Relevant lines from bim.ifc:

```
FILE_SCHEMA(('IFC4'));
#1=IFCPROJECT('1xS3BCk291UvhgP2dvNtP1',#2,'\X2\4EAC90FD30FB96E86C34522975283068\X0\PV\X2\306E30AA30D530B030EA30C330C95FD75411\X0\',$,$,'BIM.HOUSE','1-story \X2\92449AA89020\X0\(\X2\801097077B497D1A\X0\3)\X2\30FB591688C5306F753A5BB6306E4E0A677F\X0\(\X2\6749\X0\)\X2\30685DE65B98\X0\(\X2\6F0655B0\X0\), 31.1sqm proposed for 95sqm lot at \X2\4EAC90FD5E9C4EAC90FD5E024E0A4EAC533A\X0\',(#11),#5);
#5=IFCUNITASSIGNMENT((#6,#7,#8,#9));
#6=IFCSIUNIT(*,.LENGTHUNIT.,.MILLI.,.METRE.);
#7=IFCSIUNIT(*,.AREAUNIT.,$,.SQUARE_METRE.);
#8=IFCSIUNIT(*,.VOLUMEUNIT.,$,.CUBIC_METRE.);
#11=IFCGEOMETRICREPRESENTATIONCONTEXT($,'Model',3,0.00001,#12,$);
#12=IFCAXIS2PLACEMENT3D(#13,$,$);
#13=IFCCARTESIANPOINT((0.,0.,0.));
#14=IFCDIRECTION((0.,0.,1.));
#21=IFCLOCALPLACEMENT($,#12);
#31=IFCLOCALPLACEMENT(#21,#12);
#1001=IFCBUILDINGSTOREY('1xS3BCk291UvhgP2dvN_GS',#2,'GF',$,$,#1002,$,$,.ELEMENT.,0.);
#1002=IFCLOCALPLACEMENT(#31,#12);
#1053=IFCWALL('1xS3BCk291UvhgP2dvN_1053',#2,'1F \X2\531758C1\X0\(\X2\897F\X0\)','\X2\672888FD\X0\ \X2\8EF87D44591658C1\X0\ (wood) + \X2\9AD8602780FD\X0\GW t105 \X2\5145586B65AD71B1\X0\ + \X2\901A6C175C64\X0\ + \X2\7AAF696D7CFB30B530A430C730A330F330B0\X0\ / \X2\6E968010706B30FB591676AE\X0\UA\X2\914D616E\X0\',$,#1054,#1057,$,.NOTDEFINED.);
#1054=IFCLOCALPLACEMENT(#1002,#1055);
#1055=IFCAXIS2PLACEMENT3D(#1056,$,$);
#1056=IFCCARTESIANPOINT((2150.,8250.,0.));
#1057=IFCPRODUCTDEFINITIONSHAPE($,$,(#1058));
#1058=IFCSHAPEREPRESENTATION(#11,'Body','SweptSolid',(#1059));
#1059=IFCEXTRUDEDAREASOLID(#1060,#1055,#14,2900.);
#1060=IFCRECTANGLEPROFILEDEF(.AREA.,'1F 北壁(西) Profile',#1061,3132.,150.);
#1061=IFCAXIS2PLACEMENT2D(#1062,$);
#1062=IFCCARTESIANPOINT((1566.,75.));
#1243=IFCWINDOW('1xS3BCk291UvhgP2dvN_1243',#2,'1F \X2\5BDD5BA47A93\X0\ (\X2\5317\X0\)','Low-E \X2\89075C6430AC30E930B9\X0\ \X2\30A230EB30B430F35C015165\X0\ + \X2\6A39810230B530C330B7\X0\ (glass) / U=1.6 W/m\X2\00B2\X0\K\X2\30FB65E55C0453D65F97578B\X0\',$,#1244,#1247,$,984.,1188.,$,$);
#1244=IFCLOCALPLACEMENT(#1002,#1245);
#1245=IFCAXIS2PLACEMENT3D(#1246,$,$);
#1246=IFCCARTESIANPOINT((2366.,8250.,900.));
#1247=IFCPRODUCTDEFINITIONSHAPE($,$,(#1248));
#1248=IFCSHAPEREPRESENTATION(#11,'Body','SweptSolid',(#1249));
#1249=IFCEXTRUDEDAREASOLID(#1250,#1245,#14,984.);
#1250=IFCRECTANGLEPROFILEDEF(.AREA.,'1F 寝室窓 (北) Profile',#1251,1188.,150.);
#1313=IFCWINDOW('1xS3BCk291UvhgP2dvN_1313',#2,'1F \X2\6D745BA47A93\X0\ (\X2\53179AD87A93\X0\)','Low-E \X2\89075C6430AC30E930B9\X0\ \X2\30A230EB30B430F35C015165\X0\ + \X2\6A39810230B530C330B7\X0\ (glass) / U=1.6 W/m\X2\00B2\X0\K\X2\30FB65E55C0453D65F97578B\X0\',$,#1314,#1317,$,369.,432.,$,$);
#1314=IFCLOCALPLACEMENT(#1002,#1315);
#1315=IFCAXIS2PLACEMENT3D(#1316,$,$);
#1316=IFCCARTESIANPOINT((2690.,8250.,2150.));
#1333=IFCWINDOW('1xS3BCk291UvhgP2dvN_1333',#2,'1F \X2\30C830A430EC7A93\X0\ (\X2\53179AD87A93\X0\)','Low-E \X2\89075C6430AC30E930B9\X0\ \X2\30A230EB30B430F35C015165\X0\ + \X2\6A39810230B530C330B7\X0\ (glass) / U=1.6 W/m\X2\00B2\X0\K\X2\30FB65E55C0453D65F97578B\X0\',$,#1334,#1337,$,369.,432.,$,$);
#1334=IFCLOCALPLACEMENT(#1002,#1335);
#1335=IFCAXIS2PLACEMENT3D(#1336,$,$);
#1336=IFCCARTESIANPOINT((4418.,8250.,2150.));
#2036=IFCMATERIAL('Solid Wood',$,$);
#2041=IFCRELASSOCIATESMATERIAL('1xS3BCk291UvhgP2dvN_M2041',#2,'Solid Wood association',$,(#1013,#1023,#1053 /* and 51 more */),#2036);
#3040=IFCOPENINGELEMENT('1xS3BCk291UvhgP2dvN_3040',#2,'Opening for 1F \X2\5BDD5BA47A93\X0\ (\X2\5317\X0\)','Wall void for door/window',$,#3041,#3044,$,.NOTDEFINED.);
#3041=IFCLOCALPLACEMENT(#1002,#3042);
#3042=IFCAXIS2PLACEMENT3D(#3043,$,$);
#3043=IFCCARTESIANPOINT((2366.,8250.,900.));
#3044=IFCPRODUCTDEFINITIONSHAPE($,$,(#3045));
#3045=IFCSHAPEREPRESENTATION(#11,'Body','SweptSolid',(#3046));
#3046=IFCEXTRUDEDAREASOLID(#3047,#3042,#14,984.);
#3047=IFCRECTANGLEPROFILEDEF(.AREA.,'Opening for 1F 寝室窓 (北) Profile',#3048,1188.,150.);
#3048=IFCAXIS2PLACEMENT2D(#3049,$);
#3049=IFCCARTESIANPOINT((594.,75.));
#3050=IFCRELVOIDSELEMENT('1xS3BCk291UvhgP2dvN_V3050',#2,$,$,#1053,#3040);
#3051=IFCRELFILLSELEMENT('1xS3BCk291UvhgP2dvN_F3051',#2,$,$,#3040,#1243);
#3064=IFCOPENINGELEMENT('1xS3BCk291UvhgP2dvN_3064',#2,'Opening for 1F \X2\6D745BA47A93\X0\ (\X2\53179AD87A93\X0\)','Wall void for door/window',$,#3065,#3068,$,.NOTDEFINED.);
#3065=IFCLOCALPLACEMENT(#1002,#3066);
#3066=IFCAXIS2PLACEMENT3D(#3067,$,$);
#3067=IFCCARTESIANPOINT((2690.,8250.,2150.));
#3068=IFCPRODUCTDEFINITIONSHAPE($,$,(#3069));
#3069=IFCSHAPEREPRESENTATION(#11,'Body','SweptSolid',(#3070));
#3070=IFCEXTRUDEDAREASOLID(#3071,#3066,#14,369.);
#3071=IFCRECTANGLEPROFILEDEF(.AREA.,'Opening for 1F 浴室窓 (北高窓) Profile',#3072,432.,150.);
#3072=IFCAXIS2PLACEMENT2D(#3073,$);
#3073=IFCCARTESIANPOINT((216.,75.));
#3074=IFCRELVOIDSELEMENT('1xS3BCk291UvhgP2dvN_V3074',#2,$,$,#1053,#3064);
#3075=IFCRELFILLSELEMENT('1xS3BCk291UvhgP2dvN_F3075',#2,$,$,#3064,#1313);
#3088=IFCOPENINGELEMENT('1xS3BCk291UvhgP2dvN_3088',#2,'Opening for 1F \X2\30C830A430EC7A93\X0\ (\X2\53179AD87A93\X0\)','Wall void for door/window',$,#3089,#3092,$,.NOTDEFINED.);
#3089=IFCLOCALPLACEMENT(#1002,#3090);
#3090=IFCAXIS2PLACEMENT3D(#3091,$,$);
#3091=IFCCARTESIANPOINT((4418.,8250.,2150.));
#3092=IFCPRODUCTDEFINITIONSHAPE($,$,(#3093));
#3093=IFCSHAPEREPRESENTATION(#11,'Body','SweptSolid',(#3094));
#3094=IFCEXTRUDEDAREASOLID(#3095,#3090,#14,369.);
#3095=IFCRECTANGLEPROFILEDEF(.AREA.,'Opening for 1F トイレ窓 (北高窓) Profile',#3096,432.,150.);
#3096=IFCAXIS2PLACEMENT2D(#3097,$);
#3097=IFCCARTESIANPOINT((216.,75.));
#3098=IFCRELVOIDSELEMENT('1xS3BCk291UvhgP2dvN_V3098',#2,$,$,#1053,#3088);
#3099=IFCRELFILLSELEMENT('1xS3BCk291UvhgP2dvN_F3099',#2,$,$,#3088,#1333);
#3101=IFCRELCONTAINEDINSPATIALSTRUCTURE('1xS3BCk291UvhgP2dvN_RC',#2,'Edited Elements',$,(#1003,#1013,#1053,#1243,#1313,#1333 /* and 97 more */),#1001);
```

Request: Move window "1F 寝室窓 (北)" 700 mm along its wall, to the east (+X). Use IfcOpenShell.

```python
import ifcopenshell
import ifcopenshell.api.geometry
import ifcopenshell.util.placement

model = ifcopenshell.open("bim.ifc")

window = model.by_guid("1xS3BCk291UvhgP2dvN_1243")
opening = window.FillsVoids[0].RelatingOpeningElement
wall = opening.VoidsElements[0].RelatingBuildingElement

wall_matrix = ifcopenshell.util.placement.get_local_placement(wall.ObjectPlacement)
shift = wall_matrix[:3, 0] * 700.0
before = ifcopenshell.util.placement.get_local_placement(window.ObjectPlacement)[:3, 3].copy()

# The window is not placed relative to its opening, so move both.
for product in (opening, window):
    matrix = ifcopenshell.util.placement.get_local_placement(product.ObjectPlacement)
    matrix[:3, 3] += shift
    ifcopenshell.api.geometry.edit_object_placement(model, product=product, matrix=matrix, is_si=False)

after = ifcopenshell.util.placement.get_local_placement(window.ObjectPlacement)[:3, 3]
print("window moved by", (after - before).round(3) + 0.0)

model.write("bim_v2.ifc")
```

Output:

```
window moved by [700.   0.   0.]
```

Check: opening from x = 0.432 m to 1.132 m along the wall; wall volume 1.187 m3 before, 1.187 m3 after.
